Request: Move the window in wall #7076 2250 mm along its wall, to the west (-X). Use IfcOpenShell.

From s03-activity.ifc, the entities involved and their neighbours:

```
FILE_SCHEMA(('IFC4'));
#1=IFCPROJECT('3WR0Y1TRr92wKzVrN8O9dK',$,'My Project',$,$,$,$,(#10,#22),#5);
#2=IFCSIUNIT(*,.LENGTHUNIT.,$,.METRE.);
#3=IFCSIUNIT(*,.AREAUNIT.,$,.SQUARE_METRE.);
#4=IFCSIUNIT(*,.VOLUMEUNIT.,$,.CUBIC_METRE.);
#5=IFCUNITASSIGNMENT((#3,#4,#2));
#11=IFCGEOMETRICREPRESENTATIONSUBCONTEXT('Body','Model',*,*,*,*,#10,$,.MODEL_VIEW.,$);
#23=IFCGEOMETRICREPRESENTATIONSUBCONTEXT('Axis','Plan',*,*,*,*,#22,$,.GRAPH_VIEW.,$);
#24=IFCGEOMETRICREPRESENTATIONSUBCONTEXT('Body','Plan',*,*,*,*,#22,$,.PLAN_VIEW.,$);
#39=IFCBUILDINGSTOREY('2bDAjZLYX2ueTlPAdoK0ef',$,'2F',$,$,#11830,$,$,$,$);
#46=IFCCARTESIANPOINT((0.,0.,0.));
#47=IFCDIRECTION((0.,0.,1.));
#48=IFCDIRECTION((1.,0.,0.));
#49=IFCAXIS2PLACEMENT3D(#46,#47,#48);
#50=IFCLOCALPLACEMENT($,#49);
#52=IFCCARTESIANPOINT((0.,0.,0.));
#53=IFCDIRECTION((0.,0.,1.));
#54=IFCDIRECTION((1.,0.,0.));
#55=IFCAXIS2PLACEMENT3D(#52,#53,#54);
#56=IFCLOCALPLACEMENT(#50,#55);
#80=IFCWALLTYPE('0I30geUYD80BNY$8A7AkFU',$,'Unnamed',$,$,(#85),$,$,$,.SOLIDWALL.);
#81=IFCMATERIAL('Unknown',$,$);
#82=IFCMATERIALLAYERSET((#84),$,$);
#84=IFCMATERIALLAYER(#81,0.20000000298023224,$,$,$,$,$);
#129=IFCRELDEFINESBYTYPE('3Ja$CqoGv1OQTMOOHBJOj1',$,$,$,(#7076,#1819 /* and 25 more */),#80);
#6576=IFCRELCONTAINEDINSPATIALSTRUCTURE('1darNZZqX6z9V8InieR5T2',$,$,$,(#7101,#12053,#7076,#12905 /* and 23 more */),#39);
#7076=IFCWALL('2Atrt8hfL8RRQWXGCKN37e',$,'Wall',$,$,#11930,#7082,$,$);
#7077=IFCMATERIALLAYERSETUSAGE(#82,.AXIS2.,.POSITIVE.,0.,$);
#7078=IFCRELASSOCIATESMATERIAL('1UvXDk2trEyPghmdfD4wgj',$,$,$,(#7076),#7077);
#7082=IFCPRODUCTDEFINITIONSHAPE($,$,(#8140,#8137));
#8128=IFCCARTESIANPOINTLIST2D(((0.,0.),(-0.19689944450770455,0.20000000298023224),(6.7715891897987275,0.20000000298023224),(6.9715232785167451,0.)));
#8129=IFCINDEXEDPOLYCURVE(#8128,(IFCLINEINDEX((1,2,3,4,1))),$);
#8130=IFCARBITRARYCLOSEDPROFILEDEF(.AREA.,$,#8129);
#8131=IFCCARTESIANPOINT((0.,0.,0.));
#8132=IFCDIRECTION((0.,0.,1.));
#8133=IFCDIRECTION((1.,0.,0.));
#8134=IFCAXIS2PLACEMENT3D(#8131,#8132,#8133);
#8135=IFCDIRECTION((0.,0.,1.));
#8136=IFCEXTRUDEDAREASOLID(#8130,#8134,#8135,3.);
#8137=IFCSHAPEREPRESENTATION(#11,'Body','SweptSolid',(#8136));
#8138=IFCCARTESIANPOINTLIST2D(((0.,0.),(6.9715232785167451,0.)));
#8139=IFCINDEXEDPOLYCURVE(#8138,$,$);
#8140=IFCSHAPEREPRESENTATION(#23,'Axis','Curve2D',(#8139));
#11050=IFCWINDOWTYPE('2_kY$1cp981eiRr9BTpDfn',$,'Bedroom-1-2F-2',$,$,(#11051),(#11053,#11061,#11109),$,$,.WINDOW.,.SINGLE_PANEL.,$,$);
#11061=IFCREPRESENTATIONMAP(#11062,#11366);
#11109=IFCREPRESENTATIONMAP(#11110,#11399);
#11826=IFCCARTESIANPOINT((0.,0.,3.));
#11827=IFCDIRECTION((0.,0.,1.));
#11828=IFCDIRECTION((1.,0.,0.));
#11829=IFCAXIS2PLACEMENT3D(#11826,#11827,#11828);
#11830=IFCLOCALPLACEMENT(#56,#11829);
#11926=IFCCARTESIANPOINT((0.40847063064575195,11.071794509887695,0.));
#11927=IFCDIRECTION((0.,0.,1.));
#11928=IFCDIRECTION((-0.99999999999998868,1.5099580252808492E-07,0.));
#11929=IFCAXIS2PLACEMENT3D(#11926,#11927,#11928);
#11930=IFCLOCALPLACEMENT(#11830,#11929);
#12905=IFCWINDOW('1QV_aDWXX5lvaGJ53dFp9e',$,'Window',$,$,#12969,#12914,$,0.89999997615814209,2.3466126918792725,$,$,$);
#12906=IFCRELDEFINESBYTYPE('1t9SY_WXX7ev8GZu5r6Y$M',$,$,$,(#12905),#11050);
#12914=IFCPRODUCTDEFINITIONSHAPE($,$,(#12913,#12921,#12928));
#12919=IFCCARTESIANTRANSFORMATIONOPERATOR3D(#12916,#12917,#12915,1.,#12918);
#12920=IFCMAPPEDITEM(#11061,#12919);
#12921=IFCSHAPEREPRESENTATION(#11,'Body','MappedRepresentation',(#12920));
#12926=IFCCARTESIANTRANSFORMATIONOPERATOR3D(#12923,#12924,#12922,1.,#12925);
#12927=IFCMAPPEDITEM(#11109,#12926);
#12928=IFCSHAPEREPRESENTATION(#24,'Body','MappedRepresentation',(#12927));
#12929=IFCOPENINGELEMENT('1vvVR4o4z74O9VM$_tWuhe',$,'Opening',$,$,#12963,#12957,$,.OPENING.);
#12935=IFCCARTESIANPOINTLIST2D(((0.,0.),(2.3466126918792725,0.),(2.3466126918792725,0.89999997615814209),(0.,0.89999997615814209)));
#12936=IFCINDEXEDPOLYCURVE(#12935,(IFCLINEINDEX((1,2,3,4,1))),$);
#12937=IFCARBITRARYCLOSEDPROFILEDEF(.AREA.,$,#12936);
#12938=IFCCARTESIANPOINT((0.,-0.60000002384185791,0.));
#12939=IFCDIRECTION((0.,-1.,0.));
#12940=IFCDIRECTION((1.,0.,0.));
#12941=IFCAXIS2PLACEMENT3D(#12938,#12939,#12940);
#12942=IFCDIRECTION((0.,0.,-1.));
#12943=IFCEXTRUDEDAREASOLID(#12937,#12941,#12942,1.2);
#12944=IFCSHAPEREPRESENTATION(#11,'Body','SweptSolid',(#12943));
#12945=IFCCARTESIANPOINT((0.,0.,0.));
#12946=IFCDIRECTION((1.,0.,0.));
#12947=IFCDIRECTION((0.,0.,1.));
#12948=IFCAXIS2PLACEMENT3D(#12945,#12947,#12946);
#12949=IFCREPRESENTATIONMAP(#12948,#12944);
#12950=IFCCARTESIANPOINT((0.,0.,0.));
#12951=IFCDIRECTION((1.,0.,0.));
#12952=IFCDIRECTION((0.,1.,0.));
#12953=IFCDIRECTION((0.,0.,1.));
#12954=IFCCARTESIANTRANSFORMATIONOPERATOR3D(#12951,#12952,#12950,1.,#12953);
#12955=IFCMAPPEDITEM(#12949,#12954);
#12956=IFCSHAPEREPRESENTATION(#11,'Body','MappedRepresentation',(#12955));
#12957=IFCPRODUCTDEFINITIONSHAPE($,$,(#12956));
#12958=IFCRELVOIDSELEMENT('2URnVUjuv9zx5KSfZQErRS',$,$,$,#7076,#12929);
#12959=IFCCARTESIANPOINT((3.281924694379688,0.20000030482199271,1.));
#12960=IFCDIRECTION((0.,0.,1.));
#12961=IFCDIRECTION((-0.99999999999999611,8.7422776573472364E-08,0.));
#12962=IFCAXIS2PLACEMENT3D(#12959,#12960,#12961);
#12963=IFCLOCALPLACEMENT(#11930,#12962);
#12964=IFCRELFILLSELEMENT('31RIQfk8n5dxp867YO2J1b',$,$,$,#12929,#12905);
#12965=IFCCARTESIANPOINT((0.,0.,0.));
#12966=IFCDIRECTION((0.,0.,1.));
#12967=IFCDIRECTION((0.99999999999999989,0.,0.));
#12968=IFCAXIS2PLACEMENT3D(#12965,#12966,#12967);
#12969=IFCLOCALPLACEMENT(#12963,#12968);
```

```python
import ifcopenshell
import ifcopenshell.api.geometry
import ifcopenshell.util.placement
import ifcopenshell.util.unit

model = ifcopenshell.open("s03-activity.ifc")
unit_scale = ifcopenshell.util.unit.calculate_unit_scale(model)

window = model.by_guid("1QV_aDWXX5lvaGJ53dFp9e")
opening = window.FillsVoids[0].RelatingOpeningElement
wall = opening.VoidsElements[0].RelatingBuildingElement

wall_matrix = ifcopenshell.util.placement.get_local_placement(wall.ObjectPlacement)
shift = wall_matrix[:3, 0] * 2.25 / unit_scale
before = ifcopenshell.util.placement.get_local_placement(window.ObjectPlacement)[:3, 3].copy()

# The window is placed relative to its opening, so it follows when the opening moves.
matrix = ifcopenshell.util.placement.get_local_placement(opening.ObjectPlacement)
matrix[:3, 3] += shift
ifcopenshell.api.geometry.edit_object_placement(
    model, product=opening, matrix=matrix, is_si=False, should_transform_children=True
)

after = ifcopenshell.util.placement.get_local_placement(window.ObjectPlacement)[:3, 3]
print("window moved by", (after - before).round(3) + 0.0)

model.write("s03-activity-out.ifc")
```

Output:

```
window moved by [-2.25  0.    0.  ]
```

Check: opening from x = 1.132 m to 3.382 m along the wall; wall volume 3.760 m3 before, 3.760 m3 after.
